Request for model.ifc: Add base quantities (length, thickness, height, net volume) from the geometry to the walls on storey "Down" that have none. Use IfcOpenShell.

First a look at what the model holds.

```python
import ifcopenshell
import ifcopenshell.util.element
import ifcopenshell.util.unit

model = ifcopenshell.open("model.ifc")
print(model.schema)
for unit_type in ("LENGTHUNIT", "AREAUNIT", "VOLUMEUNIT"):
    print(unit_type, ifcopenshell.util.unit.calculate_unit_scale(model, unit_type))
storey = next(s for s in model.by_type("IfcBuildingStorey") if s.Name == "Down")
walls = [e for e in ifcopenshell.util.element.get_decomposition(storey) if e.is_a("IfcWall")]
for e in sorted(walls, key=lambda e: e.id()):
    print(e.id(), e.is_a(), e.Name, list(ifcopenshell.util.element.get_psets(e, qtos_only=True)), sep=" | ")
```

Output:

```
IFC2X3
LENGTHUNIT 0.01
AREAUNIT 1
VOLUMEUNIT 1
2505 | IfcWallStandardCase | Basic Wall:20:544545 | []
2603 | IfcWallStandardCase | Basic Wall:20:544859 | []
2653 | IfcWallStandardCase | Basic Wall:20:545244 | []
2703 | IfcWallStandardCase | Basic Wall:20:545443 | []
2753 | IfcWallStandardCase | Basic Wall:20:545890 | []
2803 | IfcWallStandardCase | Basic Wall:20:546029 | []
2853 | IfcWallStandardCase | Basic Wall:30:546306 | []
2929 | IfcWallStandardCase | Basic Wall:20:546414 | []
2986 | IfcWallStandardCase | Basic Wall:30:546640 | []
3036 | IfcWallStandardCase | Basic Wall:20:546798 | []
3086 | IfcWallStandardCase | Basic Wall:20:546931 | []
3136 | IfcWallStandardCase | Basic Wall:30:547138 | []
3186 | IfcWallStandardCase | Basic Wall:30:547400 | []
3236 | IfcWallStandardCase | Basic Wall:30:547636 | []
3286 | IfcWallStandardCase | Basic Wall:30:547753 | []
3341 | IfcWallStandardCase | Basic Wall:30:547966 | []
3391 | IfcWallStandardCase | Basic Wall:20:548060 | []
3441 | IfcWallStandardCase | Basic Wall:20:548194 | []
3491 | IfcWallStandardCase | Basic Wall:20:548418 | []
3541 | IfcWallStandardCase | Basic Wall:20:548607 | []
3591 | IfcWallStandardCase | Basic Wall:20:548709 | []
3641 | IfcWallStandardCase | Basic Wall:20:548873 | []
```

```python
import ifcopenshell
import ifcopenshell.api.pset
import ifcopenshell.geom
import ifcopenshell.util.element
import ifcopenshell.util.shape
import ifcopenshell.util.unit

model = ifcopenshell.open("model.ifc")
unit_scale = ifcopenshell.util.unit.calculate_unit_scale(model)
volume_scale = ifcopenshell.util.unit.calculate_unit_scale(model, "VOLUMEUNIT")
settings = ifcopenshell.geom.settings()

storey = next(s for s in model.by_type("IfcBuildingStorey") if s.Name == "Down")
walls = [e for e in ifcopenshell.util.element.get_decomposition(storey) if e.is_a("IfcWall")]

for e in sorted(walls, key=lambda e: e.id()):
    if ifcopenshell.util.element.get_psets(e, qtos_only=True, should_inherit=False):
        continue
    # Geometry comes back in metres, in the element's own axes.
    shape = ifcopenshell.geom.create_shape(settings, e)
    values = {
        "Length": ifcopenshell.util.shape.get_x(shape.geometry) / unit_scale,
        "Width": ifcopenshell.util.shape.get_y(shape.geometry) / unit_scale,
        "Height": ifcopenshell.util.shape.get_z(shape.geometry) / unit_scale,
        "NetVolume": ifcopenshell.util.shape.get_volume(shape.geometry) / volume_scale,
    }
    qto = ifcopenshell.api.pset.add_qto(model, product=e, name="BaseQuantities")
    ifcopenshell.api.pset.edit_qto(model, qto=qto, properties=values)
    print(e.id(), {k: round(v, 3) for k, v in values.items()})

model.write("model_edited.ifc")
```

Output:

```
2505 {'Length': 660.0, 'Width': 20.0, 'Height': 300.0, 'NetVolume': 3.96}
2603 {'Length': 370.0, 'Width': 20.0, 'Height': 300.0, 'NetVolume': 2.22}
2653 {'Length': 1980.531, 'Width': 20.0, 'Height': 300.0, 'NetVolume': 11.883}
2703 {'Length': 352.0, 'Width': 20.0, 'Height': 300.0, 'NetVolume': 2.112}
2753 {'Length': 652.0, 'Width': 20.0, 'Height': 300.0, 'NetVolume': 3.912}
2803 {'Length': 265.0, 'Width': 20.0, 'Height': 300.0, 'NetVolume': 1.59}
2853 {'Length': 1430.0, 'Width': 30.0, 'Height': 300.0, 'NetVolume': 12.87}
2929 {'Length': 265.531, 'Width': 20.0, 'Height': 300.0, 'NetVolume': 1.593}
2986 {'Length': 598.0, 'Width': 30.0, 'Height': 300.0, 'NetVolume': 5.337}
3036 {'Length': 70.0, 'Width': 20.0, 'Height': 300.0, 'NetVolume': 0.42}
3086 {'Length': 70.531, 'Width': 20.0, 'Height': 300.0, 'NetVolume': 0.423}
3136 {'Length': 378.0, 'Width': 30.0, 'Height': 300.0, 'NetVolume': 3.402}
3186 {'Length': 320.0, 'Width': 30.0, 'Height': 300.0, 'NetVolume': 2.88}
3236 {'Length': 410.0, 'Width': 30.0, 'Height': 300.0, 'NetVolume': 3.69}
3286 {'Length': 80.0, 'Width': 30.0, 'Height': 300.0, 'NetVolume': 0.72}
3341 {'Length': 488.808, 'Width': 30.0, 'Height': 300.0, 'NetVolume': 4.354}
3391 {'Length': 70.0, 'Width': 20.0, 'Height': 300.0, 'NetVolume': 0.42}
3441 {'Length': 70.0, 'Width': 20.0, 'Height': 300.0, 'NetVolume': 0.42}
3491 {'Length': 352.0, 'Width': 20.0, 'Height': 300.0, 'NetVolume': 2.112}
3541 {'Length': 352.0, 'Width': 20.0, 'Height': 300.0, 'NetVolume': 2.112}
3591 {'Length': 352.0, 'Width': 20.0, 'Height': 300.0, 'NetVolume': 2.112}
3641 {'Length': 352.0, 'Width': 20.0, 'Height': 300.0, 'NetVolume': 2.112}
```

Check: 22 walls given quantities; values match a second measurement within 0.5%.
